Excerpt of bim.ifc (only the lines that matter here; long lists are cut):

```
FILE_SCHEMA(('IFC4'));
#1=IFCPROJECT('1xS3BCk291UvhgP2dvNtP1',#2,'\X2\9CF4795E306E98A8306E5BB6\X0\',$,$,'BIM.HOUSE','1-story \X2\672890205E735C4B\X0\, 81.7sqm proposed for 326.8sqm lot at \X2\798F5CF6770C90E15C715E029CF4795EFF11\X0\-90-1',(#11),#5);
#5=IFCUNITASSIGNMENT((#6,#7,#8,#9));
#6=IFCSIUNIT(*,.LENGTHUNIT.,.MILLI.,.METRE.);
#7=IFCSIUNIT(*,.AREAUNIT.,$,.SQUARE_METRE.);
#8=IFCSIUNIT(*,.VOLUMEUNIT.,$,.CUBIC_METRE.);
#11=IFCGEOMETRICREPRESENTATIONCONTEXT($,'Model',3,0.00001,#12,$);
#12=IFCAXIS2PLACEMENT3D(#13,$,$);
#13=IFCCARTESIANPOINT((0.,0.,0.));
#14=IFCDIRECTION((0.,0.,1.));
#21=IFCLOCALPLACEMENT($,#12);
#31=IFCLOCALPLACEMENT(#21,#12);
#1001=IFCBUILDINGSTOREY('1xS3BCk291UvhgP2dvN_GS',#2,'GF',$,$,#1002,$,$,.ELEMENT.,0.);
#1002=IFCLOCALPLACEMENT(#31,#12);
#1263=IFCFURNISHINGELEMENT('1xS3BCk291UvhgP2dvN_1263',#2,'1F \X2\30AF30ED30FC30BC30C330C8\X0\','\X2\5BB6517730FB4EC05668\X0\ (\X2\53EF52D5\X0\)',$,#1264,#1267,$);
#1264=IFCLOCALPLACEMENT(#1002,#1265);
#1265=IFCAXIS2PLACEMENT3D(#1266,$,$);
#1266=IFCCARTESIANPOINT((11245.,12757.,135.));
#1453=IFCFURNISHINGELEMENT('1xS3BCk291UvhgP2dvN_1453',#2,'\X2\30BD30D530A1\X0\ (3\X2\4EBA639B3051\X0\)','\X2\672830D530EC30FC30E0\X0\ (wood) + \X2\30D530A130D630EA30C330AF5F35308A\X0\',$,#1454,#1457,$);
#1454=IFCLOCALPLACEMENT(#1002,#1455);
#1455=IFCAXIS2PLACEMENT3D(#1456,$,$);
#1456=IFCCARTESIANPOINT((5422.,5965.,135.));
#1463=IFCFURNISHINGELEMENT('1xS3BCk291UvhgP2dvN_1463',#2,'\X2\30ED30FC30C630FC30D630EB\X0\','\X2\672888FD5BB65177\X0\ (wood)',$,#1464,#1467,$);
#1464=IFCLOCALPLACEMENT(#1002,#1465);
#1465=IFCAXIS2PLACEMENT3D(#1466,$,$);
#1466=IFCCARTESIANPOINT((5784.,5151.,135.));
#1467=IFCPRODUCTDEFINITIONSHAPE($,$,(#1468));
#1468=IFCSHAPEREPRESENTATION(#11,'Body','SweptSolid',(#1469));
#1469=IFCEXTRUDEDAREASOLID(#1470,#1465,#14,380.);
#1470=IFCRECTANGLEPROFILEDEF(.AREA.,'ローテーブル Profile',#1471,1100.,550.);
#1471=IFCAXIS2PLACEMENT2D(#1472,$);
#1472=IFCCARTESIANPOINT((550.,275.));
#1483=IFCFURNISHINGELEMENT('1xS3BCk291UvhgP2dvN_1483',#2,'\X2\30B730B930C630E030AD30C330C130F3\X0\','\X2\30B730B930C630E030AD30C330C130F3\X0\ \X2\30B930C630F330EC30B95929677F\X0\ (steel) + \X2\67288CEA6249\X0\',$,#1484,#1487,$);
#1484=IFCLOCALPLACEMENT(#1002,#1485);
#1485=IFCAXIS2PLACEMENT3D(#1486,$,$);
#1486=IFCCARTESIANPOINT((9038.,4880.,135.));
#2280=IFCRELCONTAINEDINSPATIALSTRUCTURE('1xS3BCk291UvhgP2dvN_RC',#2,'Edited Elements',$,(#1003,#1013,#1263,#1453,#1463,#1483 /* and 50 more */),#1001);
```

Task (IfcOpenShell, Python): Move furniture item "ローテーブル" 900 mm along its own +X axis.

```python
import ifcopenshell
import ifcopenshell.api.geometry
import ifcopenshell.util.placement
import ifcopenshell.util.unit

model = ifcopenshell.open("bim.ifc")
unit_scale = ifcopenshell.util.unit.calculate_unit_scale(model)

item = model.by_guid("1xS3BCk291UvhgP2dvN_1463")
matrix = ifcopenshell.util.placement.get_local_placement(item.ObjectPlacement)
matrix[:3, 3] += matrix[:3, 0] * 0.9 / unit_scale
ifcopenshell.api.geometry.edit_object_placement(model, product=item, matrix=matrix, is_si=False)

print(ifcopenshell.util.placement.get_local_placement(item.ObjectPlacement).round(3) + 0.0)

model.write("bim_rev.ifc")
```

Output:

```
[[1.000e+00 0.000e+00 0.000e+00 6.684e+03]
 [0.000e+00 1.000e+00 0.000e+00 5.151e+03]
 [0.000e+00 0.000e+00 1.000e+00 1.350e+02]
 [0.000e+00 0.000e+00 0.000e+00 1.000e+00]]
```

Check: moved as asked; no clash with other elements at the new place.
